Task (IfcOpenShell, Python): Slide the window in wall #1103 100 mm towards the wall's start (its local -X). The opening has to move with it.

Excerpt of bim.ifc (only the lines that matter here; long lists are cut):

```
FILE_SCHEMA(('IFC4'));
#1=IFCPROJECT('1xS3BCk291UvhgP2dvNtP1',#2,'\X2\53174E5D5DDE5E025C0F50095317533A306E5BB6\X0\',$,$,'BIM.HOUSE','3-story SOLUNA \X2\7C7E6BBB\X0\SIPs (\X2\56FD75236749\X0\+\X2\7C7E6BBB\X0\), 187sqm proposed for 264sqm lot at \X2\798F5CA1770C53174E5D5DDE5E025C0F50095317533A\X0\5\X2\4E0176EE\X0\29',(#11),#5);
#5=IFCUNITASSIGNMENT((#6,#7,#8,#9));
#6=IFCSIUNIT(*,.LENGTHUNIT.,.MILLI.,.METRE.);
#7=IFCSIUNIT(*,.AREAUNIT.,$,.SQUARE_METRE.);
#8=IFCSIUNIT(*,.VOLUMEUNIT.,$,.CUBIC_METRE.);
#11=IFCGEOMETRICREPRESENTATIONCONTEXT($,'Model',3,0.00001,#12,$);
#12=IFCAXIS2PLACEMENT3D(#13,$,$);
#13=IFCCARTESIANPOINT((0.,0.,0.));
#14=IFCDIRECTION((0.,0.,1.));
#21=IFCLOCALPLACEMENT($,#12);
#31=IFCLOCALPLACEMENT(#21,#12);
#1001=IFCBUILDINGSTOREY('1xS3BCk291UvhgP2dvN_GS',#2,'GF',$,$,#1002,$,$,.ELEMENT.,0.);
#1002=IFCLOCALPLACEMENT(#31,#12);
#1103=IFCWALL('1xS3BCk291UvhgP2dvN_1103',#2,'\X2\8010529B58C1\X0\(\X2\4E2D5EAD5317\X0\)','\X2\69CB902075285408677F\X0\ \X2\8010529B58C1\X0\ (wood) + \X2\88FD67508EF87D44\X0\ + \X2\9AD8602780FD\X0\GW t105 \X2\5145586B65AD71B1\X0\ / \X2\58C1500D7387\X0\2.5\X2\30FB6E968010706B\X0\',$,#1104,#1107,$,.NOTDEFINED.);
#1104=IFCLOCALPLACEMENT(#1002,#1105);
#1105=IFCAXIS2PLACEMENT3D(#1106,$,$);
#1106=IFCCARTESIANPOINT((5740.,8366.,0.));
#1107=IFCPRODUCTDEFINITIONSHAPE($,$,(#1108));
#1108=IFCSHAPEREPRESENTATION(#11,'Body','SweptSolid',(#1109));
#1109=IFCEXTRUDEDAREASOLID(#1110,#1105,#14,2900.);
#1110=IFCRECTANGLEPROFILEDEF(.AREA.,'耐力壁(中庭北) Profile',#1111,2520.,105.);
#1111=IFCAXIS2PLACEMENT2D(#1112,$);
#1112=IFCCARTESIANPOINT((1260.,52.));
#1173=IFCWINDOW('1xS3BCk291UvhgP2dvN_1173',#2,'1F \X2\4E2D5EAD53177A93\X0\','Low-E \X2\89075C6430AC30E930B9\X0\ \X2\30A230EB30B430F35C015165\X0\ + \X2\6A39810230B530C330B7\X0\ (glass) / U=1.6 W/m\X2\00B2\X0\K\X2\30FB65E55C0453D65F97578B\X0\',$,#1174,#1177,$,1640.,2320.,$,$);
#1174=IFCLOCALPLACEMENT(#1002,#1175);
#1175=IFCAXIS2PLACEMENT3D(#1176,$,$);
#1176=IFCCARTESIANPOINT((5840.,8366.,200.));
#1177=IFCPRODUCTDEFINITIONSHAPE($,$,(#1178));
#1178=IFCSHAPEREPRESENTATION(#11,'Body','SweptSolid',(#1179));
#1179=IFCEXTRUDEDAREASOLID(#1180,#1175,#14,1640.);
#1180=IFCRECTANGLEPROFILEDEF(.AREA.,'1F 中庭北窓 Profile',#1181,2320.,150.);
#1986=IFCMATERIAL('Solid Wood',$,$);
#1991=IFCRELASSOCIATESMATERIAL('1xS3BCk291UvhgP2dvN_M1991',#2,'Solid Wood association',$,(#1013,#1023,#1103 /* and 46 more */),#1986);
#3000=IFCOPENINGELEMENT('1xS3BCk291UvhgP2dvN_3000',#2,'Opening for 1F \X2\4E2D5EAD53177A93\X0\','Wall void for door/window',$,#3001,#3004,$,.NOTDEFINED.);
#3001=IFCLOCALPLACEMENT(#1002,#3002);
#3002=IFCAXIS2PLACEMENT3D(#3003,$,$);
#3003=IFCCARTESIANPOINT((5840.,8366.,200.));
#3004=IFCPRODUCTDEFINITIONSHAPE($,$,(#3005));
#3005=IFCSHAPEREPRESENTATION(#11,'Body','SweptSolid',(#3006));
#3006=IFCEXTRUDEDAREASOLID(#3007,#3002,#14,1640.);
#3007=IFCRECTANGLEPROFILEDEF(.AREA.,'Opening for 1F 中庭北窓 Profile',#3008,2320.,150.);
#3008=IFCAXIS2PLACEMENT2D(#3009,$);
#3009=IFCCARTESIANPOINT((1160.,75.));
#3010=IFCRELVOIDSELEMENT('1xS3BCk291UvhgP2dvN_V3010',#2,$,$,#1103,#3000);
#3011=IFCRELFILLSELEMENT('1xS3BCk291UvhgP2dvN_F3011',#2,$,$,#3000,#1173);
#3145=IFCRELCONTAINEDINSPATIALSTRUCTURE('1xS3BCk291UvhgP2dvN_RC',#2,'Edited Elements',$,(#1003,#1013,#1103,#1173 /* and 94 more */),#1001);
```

```python
import ifcopenshell
import ifcopenshell.api.geometry
import ifcopenshell.util.placement
import ifcopenshell.util.unit

model = ifcopenshell.open("bim.ifc")
unit_scale = ifcopenshell.util.unit.calculate_unit_scale(model)

window = model.by_guid("1xS3BCk291UvhgP2dvN_1173")
opening = window.FillsVoids[0].RelatingOpeningElement
wall = opening.VoidsElements[0].RelatingBuildingElement

wall_matrix = ifcopenshell.util.placement.get_local_placement(wall.ObjectPlacement)
shift = wall_matrix[:3, 0] * -0.1 / unit_scale
before = ifcopenshell.util.placement.get_local_placement(window.ObjectPlacement)[:3, 3].copy()

# The window is not placed relative to its opening, so move both.
for product in (opening, window):
    matrix = ifcopenshell.util.placement.get_local_placement(product.ObjectPlacement)
    matrix[:3, 3] += shift
    ifcopenshell.api.geometry.edit_object_placement(model, product=product, matrix=matrix, is_si=False)

after = ifcopenshell.util.placement.get_local_placement(window.ObjectPlacement)[:3, 3]
print("window moved by", (after - before).round(3) + 0.0)

model.write("bim_updated.ifc")
```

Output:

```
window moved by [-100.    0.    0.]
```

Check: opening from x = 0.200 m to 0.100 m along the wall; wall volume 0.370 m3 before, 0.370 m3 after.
